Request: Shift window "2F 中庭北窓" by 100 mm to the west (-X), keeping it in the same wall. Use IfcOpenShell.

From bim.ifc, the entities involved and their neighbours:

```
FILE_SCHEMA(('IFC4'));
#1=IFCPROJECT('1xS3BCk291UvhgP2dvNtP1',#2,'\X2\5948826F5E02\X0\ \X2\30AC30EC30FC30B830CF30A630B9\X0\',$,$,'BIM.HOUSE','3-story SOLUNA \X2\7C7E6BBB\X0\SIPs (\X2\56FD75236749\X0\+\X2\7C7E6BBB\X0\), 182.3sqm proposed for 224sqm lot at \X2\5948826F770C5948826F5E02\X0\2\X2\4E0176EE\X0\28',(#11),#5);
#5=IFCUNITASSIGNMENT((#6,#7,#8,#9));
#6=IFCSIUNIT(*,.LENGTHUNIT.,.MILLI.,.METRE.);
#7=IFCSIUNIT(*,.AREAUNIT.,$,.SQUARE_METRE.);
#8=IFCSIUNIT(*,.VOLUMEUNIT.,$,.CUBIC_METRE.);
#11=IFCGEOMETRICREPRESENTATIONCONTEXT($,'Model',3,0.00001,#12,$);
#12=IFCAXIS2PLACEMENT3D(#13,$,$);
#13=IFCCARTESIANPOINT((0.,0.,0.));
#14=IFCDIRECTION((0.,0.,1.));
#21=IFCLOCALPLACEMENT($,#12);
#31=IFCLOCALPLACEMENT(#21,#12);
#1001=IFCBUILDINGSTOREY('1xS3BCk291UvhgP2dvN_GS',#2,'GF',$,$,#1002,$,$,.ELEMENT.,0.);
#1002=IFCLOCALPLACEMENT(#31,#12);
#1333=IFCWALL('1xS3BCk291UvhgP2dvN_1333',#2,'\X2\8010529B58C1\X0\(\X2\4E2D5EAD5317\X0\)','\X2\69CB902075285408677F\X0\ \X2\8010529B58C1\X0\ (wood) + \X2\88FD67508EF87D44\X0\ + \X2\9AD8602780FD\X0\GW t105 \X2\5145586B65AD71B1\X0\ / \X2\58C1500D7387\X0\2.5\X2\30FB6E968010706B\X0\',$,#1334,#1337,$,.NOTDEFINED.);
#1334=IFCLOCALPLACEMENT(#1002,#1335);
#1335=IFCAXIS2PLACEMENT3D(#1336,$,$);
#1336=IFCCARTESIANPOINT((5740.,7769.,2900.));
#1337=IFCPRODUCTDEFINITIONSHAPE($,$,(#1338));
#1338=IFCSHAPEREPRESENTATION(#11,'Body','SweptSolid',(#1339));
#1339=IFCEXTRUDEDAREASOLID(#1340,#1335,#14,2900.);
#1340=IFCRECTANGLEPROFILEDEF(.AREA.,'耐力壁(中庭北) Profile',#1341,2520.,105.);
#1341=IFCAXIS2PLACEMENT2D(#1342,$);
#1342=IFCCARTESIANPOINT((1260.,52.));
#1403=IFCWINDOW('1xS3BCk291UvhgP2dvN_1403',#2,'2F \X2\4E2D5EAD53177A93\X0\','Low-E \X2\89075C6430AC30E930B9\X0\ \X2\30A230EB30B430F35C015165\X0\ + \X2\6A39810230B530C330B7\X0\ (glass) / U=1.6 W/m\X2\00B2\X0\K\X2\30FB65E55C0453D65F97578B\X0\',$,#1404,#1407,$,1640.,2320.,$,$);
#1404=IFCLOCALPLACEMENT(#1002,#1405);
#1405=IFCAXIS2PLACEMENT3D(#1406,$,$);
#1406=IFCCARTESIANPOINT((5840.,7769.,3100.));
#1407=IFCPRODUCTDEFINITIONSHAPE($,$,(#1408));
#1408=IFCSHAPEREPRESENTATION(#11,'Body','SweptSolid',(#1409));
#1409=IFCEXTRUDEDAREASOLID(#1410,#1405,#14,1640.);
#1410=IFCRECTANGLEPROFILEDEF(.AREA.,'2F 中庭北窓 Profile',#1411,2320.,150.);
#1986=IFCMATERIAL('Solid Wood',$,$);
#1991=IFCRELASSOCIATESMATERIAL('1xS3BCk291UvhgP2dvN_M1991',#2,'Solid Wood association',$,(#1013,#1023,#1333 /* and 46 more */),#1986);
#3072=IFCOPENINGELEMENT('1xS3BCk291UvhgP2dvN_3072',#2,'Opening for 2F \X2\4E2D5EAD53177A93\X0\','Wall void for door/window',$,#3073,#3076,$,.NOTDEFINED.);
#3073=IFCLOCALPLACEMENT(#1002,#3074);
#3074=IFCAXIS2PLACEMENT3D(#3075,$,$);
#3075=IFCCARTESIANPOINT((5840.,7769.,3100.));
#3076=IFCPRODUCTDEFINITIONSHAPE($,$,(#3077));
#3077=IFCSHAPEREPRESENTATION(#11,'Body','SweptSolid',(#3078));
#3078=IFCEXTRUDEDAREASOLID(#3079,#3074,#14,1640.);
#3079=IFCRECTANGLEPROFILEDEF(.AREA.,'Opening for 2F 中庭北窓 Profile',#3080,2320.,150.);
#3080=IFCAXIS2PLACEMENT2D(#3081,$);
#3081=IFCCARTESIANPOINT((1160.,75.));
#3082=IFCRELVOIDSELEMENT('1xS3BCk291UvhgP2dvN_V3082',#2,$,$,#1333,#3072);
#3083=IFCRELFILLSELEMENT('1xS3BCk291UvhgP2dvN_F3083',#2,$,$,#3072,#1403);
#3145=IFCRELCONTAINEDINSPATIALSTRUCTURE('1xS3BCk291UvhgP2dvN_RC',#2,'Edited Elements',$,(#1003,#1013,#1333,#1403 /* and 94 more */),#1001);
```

```python
import ifcopenshell
import ifcopenshell.api.geometry
import ifcopenshell.util.placement
import ifcopenshell.util.unit

model = ifcopenshell.open("bim.ifc")
unit_scale = ifcopenshell.util.unit.calculate_unit_scale(model)

window = model.by_guid("1xS3BCk291UvhgP2dvN_1403")
opening = window.FillsVoids[0].RelatingOpeningElement
wall = opening.VoidsElements[0].RelatingBuildingElement

wall_matrix = ifcopenshell.util.placement.get_local_placement(wall.ObjectPlacement)
shift = wall_matrix[:3, 0] * -0.1 / unit_scale
before = ifcopenshell.util.placement.get_local_placement(window.ObjectPlacement)[:3, 3].copy()

# The window is not placed relative to its opening, so move both.
for product in (opening, window):
    matrix = ifcopenshell.util.placement.get_local_placement(product.ObjectPlacement)
    matrix[:3, 3] += shift
    ifcopenshell.api.geometry.edit_object_placement(model, product=product, matrix=matrix, is_si=False)

after = ifcopenshell.util.placement.get_local_placement(window.ObjectPlacement)[:3, 3]
print("window moved by", (after - before).round(3) + 0.0)

model.write("bim_edited.ifc")
```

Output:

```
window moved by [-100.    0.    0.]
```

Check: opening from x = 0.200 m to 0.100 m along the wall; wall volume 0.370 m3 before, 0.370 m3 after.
